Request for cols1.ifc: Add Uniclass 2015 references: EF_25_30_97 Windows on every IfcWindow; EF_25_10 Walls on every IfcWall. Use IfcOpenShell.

First a look at what the model holds.

```python
import ifcopenshell

model = ifcopenshell.open("cols1.ifc")
print(model.schema)
print("classifications:", [c.Name for c in model.by_type("IfcClassification")])
for ifc_class in ("IfcDoor", "IfcRoof", "IfcStair", "IfcWall", "IfcWindow"):
    print(ifc_class, len(model.by_type(ifc_class)))
```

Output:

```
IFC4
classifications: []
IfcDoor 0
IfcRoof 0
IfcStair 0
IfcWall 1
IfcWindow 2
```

```python
import ifcopenshell
import ifcopenshell.api.classification

model = ifcopenshell.open("cols1.ifc")

system = ifcopenshell.api.classification.add_classification(model, classification="Uniclass 2015")

codes = {
    "IfcWindow": ("EF_25_30_97", "Windows"),
    "IfcWall": ("EF_25_10", "Walls"),
}
for ifc_class, (code, name) in codes.items():
    products = model.by_type(ifc_class)
    ifcopenshell.api.classification.add_reference(
        model, products=products, classification=system, identification=code, name=name
    )
    print(code, len(products))

model.write("cols1_edited.ifc")
```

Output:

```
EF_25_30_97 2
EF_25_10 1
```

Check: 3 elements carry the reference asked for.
